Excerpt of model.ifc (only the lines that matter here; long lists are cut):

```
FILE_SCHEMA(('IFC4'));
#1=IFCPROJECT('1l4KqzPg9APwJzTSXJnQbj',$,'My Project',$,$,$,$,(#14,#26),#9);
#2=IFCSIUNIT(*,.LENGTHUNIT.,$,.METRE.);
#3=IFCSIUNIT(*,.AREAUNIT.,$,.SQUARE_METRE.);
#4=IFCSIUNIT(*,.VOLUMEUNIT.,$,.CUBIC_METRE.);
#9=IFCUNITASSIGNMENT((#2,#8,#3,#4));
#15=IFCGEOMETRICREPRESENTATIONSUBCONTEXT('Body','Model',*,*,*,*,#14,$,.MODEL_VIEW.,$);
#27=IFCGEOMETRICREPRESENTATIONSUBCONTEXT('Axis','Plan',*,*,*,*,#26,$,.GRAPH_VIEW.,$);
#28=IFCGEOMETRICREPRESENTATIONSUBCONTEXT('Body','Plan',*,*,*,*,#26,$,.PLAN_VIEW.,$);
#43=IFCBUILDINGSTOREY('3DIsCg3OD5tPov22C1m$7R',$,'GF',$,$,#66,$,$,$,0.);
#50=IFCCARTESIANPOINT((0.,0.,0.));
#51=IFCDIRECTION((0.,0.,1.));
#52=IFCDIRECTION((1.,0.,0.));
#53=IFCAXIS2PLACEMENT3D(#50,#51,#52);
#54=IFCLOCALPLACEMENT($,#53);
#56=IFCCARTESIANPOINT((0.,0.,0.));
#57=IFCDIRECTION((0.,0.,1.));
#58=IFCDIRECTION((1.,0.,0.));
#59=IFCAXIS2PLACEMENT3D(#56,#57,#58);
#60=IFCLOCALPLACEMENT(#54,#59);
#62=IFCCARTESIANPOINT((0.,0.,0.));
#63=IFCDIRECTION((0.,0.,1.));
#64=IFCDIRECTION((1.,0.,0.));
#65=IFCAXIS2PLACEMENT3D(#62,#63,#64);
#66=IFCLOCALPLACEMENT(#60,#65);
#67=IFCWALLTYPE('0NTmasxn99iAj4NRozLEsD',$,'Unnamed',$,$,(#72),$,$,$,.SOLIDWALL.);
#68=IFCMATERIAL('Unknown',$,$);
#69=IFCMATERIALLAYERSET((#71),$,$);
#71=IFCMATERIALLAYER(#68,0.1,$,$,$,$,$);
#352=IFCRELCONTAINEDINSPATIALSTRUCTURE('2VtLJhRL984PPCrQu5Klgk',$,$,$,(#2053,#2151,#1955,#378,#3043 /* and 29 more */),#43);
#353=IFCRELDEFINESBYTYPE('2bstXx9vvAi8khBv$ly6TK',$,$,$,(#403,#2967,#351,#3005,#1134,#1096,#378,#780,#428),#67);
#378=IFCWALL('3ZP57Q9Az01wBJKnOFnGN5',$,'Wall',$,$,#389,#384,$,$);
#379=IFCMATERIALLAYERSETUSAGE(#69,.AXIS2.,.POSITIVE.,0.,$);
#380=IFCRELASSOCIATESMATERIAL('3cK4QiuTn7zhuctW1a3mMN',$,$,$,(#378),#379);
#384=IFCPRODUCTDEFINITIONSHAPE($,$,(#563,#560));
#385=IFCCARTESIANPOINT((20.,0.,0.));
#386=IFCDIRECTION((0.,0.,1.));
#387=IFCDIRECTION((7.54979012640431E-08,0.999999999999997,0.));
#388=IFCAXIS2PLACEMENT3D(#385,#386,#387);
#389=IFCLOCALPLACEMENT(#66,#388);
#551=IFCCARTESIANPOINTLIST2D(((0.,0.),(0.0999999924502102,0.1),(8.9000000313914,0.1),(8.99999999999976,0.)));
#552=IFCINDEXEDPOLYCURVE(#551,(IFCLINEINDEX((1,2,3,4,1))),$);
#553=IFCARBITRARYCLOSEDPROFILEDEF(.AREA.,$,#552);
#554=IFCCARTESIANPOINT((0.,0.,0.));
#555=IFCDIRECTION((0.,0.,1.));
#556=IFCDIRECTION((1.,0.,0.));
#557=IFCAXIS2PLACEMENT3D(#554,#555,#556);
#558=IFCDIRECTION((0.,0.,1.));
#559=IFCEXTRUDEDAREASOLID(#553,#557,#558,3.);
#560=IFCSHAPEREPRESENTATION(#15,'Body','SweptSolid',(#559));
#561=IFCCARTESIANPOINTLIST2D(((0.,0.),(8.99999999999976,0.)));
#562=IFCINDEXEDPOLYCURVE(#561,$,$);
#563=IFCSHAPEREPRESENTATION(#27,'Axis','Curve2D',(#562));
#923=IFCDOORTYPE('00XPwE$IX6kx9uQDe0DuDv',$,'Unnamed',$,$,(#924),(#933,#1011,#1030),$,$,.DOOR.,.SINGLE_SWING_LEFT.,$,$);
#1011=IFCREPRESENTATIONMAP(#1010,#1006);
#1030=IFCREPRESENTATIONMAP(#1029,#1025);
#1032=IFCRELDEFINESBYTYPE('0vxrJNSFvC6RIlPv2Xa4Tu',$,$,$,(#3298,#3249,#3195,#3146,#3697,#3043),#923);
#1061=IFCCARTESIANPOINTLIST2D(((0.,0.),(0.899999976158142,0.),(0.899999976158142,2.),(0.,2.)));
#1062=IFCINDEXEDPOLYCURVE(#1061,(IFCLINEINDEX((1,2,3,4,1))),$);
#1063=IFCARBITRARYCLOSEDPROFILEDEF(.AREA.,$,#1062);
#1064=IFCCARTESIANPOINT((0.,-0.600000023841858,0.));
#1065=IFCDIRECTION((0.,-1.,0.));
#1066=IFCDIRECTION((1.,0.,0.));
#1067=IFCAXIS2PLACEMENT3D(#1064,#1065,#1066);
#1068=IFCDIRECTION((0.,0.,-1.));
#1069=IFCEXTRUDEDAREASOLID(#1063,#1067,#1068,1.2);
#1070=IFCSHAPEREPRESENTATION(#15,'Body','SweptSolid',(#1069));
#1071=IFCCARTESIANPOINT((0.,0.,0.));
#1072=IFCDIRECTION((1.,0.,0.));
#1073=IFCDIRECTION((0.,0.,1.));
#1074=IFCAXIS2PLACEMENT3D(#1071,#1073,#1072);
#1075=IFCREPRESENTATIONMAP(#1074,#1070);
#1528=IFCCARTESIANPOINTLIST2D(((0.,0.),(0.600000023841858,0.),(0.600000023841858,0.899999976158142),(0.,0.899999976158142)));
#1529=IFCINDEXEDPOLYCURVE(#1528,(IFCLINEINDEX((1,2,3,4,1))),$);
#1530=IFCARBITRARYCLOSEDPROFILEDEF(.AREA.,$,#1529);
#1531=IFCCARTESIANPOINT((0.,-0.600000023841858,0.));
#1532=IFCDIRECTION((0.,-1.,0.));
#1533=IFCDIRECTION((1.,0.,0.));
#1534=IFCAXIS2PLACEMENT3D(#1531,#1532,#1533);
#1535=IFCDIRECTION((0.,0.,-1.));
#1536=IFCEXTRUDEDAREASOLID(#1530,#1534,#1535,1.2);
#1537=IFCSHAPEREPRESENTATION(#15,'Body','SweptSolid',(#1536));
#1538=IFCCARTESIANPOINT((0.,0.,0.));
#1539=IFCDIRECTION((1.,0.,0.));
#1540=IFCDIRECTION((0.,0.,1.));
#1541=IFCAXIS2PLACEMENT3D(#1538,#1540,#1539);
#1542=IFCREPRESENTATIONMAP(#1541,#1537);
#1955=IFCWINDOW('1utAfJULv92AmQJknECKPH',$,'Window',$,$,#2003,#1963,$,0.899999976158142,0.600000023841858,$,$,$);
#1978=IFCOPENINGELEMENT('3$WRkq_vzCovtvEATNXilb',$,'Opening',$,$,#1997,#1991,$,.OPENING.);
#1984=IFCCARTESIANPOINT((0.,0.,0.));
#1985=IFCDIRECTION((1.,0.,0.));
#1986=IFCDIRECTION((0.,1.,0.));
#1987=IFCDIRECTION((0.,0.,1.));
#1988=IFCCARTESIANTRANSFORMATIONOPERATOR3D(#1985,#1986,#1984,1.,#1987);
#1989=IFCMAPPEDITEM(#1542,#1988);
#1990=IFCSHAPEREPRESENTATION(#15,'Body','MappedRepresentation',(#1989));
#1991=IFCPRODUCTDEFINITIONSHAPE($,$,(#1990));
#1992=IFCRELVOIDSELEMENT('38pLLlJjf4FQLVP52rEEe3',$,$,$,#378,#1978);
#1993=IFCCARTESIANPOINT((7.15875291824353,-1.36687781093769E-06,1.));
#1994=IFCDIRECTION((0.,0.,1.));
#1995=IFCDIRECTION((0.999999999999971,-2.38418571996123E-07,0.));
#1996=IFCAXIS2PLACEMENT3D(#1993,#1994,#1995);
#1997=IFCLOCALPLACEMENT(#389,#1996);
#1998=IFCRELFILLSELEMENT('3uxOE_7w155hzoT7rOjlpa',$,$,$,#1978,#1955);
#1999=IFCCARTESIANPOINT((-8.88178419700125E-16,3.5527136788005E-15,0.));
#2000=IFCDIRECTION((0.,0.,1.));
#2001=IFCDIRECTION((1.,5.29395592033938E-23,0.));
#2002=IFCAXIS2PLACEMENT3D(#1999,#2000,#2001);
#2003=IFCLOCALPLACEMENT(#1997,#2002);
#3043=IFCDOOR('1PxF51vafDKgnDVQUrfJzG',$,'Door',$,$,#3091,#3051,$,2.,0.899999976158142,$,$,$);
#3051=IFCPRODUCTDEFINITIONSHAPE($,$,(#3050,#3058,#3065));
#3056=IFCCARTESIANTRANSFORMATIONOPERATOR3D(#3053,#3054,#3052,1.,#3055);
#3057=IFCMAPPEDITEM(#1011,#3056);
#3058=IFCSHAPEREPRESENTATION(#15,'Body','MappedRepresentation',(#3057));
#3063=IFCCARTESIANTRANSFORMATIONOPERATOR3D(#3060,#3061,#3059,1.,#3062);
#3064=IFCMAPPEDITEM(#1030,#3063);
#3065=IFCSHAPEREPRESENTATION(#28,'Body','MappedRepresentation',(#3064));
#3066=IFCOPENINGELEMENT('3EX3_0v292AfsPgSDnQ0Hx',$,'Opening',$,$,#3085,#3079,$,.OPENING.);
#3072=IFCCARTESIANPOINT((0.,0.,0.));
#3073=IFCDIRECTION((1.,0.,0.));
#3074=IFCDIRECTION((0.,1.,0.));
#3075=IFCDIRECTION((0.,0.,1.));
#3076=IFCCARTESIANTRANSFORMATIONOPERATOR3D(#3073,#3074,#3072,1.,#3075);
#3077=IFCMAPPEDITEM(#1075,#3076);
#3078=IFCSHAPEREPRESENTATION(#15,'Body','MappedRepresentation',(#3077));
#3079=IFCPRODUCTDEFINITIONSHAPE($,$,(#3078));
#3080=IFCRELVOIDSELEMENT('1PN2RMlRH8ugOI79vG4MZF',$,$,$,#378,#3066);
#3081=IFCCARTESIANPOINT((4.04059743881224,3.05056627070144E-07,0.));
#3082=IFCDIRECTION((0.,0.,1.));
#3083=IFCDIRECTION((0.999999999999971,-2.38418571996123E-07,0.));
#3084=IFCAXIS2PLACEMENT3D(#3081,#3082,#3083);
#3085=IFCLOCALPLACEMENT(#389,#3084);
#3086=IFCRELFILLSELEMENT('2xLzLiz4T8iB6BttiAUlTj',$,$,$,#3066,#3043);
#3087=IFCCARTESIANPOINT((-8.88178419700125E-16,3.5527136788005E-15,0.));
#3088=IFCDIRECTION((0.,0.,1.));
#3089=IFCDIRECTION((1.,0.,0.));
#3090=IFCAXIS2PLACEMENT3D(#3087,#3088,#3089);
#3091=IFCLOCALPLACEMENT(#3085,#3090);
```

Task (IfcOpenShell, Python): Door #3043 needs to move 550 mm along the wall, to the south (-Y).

```python
import ifcopenshell
import ifcopenshell.api.geometry
import ifcopenshell.util.placement

model = ifcopenshell.open("model.ifc")

door = model.by_guid("1PxF51vafDKgnDVQUrfJzG")
opening = door.FillsVoids[0].RelatingOpeningElement
wall = opening.VoidsElements[0].RelatingBuildingElement

wall_matrix = ifcopenshell.util.placement.get_local_placement(wall.ObjectPlacement)
shift = wall_matrix[:3, 0] * -0.55
before = ifcopenshell.util.placement.get_local_placement(door.ObjectPlacement)[:3, 3].copy()

# The door is placed relative to its opening, so it follows when the opening moves.
matrix = ifcopenshell.util.placement.get_local_placement(opening.ObjectPlacement)
matrix[:3, 3] += shift
ifcopenshell.api.geometry.edit_object_placement(
    model, product=opening, matrix=matrix, is_si=False, should_transform_children=True
)

after = ifcopenshell.util.placement.get_local_placement(door.ObjectPlacement)[:3, 3]
print("door moved by", (after - before).round(3) + 0.0)

model.write("model_updated.ifc")
```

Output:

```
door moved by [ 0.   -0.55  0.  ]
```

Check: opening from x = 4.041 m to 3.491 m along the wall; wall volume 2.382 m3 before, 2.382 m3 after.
